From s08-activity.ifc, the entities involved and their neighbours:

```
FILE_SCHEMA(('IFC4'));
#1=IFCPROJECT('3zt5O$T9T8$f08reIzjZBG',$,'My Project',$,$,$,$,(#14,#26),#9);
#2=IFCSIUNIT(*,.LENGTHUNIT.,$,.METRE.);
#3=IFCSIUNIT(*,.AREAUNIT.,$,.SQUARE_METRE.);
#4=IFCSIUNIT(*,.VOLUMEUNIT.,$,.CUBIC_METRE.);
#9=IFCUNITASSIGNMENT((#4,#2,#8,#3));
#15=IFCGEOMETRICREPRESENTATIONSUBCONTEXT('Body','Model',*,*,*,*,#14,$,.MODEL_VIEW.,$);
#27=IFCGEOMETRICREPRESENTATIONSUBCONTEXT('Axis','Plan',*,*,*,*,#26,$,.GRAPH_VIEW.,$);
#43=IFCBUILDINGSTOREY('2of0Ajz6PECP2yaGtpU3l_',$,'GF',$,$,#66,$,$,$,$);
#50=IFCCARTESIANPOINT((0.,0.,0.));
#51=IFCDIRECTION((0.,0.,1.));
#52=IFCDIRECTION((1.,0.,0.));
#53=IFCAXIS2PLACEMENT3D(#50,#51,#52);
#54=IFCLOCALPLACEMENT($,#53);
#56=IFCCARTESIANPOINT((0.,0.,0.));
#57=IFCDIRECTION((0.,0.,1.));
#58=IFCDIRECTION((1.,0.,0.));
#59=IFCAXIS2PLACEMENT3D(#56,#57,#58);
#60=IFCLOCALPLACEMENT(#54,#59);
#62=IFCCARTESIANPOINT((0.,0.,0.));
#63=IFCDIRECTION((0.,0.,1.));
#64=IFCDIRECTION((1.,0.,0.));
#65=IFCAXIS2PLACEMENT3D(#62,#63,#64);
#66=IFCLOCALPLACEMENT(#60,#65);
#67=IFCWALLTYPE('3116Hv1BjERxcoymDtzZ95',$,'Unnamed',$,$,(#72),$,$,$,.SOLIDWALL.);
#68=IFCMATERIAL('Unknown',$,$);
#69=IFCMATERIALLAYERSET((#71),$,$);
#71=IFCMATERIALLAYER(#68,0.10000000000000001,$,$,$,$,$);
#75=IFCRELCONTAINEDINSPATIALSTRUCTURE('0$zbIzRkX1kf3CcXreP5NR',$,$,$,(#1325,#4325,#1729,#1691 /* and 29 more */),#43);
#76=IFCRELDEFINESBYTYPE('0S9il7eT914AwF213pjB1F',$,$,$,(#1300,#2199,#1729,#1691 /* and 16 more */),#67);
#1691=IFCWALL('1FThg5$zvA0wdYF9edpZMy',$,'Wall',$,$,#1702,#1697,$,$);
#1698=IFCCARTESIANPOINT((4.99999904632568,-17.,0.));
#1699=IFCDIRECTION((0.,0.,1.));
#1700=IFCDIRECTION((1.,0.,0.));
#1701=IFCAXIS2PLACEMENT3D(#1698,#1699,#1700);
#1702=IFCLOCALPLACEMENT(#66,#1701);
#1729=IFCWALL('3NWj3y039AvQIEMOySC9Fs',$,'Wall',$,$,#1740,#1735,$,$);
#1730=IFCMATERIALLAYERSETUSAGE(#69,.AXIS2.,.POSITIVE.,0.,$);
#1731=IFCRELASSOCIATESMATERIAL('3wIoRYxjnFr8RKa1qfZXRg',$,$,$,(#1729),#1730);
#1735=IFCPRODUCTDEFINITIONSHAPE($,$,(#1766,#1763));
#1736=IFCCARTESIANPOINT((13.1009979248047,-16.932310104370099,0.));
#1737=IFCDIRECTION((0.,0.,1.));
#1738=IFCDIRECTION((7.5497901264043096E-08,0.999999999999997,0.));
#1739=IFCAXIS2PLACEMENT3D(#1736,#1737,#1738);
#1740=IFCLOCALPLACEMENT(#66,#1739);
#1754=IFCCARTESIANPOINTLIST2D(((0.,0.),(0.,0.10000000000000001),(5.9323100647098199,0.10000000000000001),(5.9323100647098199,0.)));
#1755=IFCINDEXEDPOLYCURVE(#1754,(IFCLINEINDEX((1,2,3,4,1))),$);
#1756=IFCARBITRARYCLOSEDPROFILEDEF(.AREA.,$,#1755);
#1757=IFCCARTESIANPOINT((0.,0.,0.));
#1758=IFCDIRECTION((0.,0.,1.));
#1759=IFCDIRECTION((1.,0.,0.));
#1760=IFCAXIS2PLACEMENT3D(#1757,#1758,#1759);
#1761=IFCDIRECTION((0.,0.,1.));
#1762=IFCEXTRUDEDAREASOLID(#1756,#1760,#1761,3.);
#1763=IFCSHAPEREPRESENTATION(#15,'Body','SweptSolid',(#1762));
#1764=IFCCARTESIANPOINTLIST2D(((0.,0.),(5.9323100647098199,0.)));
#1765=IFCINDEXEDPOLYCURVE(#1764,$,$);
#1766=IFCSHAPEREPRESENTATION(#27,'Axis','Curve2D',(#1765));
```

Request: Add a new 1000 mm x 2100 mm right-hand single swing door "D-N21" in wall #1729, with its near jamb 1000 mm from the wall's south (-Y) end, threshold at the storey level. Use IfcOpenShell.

```python
import numpy as np
import ifcopenshell
import ifcopenshell.api.feature
import ifcopenshell.api.geometry
import ifcopenshell.api.root
import ifcopenshell.api.spatial
import ifcopenshell.geom
import ifcopenshell.util.element
import ifcopenshell.util.placement
import ifcopenshell.util.representation
import ifcopenshell.util.shape
import ifcopenshell.util.unit

model = ifcopenshell.open("s08-activity.ifc")
unit_scale = ifcopenshell.util.unit.calculate_unit_scale(model)
settings = ifcopenshell.geom.settings()


def volume(element):
    """Net volume in cubic metres, openings subtracted."""
    shape = ifcopenshell.geom.create_shape(settings, element)
    return ifcopenshell.util.shape.get_volume(shape.geometry)


wall = model.by_id(1729)
storey = ifcopenshell.util.element.get_container(wall, ifc_class="IfcBuildingStorey")
context = ifcopenshell.util.representation.get_context(model, "Model", "Body", "MODEL_VIEW")
before = volume(wall)

width, height, from_end, sill = 1, 2.1, 1, 0.0  # metres

# The wall runs along its own X axis, and the end named is its -X end.
wall_shape = ifcopenshell.geom.create_shape(settings, wall)
x, y, z = ifcopenshell.util.shape.get_vertices(wall_shape.geometry).T
start = x.min() + from_end
face, thickness = float(y.min()), float(y.max() - y.min())
wall_matrix = ifcopenshell.util.placement.get_local_placement(wall.ObjectPlacement)
level = ifcopenshell.util.placement.get_local_placement(storey.ObjectPlacement)[2, 3]


def in_wall(x, y):
    """Placement at x, y metres in the wall's axes, at sill height."""
    matrix = wall_matrix.copy()
    matrix[:, 3] = wall_matrix @ np.array([x / unit_scale, y / unit_scale, 0.0, 1.0])
    matrix[2, 3] = level + sill / unit_scale
    return matrix


# Opening: a box that overshoots both wall faces by 50 mm.
opening = ifcopenshell.api.root.create_entity(model, ifc_class="IfcOpeningElement", predefined_type="OPENING")
box = ifcopenshell.api.geometry.add_wall_representation(
    model, context=context, length=width, height=height, thickness=thickness + 0.1
)
ifcopenshell.api.geometry.assign_representation(model, product=opening, representation=box)
ifcopenshell.api.geometry.edit_object_placement(model, product=opening, matrix=in_wall(start, face - 0.05), is_si=False)
ifcopenshell.api.feature.add_feature(model, feature=opening, element=wall)

door = ifcopenshell.api.root.create_entity(model, ifc_class="IfcDoor", name="D-N21", predefined_type="DOOR")
door.OverallWidth, door.OverallHeight = width / unit_scale, height / unit_scale
door.OperationType = "SINGLE_SWING_RIGHT"
body = ifcopenshell.api.geometry.add_door_representation(
    model,
    context=context,
    overall_width=door.OverallWidth,
    overall_height=door.OverallHeight,
    operation_type="SINGLE_SWING_RIGHT",
    lining_properties={"LiningDepth": thickness / unit_scale, "ThresholdDepth": thickness / unit_scale},
)
ifcopenshell.api.geometry.assign_representation(model, product=door, representation=body)
ifcopenshell.api.spatial.assign_container(model, products=[door], relating_structure=storey)
ifcopenshell.api.feature.add_filling(model, opening=opening, element=door)

# The lining spans the wall, so the door starts at the wall face.
ifcopenshell.api.geometry.edit_object_placement(model, product=door, matrix=in_wall(start, face), is_si=False)

after = volume(wall)

print(f"wall volume {before:.3f} -> {after:.3f} m3")

model.write("s08-activity_v2.ifc")
```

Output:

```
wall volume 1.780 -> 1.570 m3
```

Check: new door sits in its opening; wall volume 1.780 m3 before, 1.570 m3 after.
